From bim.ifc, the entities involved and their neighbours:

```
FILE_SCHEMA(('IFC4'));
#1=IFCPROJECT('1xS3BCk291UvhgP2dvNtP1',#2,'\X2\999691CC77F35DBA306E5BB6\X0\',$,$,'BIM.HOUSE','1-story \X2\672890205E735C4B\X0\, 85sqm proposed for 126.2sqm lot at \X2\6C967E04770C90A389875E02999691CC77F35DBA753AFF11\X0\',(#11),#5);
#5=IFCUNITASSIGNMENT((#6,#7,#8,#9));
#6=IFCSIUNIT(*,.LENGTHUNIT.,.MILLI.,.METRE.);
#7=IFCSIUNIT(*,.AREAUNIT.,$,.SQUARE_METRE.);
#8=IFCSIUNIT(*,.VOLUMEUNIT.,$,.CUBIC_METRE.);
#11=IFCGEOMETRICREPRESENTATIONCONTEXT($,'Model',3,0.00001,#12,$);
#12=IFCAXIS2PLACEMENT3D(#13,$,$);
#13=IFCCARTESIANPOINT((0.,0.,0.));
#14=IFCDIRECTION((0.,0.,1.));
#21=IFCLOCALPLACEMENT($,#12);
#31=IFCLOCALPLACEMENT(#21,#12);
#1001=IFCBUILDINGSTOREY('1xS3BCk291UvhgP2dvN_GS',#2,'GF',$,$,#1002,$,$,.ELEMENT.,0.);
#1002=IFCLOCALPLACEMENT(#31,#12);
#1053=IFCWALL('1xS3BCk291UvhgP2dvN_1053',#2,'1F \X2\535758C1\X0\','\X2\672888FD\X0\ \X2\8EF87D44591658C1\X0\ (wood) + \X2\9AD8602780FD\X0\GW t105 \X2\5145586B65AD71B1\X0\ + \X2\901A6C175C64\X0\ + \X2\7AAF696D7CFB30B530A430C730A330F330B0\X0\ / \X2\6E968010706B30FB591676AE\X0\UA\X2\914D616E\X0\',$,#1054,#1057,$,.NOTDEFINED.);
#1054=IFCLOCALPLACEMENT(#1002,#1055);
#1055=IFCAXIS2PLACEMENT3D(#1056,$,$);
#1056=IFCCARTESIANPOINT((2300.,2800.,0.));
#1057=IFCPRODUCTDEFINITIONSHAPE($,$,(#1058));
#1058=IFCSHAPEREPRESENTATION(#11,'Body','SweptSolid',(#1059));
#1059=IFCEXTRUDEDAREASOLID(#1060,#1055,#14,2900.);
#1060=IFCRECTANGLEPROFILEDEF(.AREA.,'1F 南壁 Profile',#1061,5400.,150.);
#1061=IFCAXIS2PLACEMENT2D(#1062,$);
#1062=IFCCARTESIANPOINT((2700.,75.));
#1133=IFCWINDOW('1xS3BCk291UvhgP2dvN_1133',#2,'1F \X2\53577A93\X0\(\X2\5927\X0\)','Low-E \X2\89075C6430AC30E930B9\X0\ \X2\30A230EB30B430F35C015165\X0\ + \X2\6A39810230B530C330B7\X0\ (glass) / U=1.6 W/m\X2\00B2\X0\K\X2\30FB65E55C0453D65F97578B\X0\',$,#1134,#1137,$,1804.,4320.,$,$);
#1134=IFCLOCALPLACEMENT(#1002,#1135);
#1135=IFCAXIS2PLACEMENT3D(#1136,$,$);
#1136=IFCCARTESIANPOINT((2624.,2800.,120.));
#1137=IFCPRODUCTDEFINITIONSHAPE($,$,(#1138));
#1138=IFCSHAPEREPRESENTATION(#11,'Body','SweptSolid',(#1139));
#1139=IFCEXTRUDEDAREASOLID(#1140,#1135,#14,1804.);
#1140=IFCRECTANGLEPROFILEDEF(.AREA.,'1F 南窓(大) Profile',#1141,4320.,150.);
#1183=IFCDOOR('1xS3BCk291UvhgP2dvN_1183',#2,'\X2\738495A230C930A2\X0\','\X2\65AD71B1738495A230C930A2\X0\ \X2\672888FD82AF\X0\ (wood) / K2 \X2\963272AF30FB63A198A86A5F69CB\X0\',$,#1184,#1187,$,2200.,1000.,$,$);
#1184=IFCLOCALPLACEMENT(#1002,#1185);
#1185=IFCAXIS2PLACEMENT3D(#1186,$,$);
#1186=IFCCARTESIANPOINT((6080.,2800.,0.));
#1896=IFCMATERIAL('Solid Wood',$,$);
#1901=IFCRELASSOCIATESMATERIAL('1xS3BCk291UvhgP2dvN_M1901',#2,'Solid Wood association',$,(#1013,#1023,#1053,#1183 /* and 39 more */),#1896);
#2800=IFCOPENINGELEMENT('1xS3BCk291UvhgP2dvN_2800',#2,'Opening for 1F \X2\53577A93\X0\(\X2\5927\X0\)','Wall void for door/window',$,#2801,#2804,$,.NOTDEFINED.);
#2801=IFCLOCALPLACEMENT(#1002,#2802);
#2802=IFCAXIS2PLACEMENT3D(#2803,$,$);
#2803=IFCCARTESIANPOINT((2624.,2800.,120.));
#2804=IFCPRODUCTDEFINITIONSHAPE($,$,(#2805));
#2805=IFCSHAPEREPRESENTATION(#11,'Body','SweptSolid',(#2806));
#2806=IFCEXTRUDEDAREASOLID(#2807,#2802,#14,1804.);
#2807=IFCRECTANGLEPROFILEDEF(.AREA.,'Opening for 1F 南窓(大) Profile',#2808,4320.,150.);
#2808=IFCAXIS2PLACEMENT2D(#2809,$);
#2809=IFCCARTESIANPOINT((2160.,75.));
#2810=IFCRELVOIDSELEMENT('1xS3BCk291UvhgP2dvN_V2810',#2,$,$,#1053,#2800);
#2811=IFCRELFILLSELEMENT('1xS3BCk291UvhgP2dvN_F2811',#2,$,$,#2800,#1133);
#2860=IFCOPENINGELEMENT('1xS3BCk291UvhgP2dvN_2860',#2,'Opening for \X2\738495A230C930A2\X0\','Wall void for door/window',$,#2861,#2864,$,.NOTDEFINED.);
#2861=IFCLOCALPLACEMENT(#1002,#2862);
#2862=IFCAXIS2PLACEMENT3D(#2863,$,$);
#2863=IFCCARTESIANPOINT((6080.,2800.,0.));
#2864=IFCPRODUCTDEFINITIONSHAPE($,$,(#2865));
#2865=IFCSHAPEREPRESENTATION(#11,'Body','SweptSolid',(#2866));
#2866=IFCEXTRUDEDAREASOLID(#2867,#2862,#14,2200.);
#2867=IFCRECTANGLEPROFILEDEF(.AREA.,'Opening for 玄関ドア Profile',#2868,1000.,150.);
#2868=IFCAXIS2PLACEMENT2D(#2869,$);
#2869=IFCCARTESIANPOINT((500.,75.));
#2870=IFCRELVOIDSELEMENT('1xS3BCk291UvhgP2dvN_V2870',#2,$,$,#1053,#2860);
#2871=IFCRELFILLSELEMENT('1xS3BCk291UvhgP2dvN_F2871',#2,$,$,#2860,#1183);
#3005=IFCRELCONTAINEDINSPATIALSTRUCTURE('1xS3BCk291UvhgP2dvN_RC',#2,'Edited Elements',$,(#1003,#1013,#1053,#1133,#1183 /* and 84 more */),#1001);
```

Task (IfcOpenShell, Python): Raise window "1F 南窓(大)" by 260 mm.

```python
import numpy as np
import ifcopenshell
import ifcopenshell.api.geometry
import ifcopenshell.util.placement
import ifcopenshell.util.unit

model = ifcopenshell.open("bim.ifc")
unit_scale = ifcopenshell.util.unit.calculate_unit_scale(model)

window = model.by_guid("1xS3BCk291UvhgP2dvN_1133")
opening = window.FillsVoids[0].RelatingOpeningElement
dz = 0.26 / unit_scale

shift = np.array([0.0, 0.0, dz])
# The window is not placed relative to its opening, so move both.
for product in (opening, window):
    matrix = ifcopenshell.util.placement.get_local_placement(product.ObjectPlacement)
    matrix[:3, 3] += shift
    ifcopenshell.api.geometry.edit_object_placement(model, product=product, matrix=matrix, is_si=False)

print(f"moved by {dz * unit_scale:+.3f} m")

model.write("bim_edited.ifc")
```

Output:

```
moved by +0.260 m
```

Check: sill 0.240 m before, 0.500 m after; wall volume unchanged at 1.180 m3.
